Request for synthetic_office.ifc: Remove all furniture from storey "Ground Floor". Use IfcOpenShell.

First a look at what the model holds.

```python
import ifcopenshell
import ifcopenshell.util.element

model = ifcopenshell.open("synthetic_office.ifc")
print(model.schema)
storey = next(s for s in model.by_type("IfcBuildingStorey") if s.Name == "Ground Floor")
furniture = [e for e in ifcopenshell.util.element.get_decomposition(storey) if e.is_a("IfcFurnishingElement")]
seen = {}
for e in furniture:
    element_type = ifcopenshell.util.element.get_type(e)
    name = element_type.Name if element_type not in (None, e) else None
    seen[name] = seen.get(name, 0) + 1
for name, count in sorted(seen.items(), key=str):
    print(count, "x", name)
```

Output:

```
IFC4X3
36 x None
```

```python
import ifcopenshell
import ifcopenshell.api.root
import ifcopenshell.util.element

model = ifcopenshell.open("synthetic_office.ifc")

storey = next(s for s in model.by_type("IfcBuildingStorey") if s.Name == "Ground Floor")
furniture = [e for e in ifcopenshell.util.element.get_decomposition(storey) if e.is_a("IfcFurnishingElement")]

for e in furniture:
    ifcopenshell.api.root.remove_product(model, product=e)
print(len(furniture), "removed")

model.write("synthetic_office_edited.ifc")
```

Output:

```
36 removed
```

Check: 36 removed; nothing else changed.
